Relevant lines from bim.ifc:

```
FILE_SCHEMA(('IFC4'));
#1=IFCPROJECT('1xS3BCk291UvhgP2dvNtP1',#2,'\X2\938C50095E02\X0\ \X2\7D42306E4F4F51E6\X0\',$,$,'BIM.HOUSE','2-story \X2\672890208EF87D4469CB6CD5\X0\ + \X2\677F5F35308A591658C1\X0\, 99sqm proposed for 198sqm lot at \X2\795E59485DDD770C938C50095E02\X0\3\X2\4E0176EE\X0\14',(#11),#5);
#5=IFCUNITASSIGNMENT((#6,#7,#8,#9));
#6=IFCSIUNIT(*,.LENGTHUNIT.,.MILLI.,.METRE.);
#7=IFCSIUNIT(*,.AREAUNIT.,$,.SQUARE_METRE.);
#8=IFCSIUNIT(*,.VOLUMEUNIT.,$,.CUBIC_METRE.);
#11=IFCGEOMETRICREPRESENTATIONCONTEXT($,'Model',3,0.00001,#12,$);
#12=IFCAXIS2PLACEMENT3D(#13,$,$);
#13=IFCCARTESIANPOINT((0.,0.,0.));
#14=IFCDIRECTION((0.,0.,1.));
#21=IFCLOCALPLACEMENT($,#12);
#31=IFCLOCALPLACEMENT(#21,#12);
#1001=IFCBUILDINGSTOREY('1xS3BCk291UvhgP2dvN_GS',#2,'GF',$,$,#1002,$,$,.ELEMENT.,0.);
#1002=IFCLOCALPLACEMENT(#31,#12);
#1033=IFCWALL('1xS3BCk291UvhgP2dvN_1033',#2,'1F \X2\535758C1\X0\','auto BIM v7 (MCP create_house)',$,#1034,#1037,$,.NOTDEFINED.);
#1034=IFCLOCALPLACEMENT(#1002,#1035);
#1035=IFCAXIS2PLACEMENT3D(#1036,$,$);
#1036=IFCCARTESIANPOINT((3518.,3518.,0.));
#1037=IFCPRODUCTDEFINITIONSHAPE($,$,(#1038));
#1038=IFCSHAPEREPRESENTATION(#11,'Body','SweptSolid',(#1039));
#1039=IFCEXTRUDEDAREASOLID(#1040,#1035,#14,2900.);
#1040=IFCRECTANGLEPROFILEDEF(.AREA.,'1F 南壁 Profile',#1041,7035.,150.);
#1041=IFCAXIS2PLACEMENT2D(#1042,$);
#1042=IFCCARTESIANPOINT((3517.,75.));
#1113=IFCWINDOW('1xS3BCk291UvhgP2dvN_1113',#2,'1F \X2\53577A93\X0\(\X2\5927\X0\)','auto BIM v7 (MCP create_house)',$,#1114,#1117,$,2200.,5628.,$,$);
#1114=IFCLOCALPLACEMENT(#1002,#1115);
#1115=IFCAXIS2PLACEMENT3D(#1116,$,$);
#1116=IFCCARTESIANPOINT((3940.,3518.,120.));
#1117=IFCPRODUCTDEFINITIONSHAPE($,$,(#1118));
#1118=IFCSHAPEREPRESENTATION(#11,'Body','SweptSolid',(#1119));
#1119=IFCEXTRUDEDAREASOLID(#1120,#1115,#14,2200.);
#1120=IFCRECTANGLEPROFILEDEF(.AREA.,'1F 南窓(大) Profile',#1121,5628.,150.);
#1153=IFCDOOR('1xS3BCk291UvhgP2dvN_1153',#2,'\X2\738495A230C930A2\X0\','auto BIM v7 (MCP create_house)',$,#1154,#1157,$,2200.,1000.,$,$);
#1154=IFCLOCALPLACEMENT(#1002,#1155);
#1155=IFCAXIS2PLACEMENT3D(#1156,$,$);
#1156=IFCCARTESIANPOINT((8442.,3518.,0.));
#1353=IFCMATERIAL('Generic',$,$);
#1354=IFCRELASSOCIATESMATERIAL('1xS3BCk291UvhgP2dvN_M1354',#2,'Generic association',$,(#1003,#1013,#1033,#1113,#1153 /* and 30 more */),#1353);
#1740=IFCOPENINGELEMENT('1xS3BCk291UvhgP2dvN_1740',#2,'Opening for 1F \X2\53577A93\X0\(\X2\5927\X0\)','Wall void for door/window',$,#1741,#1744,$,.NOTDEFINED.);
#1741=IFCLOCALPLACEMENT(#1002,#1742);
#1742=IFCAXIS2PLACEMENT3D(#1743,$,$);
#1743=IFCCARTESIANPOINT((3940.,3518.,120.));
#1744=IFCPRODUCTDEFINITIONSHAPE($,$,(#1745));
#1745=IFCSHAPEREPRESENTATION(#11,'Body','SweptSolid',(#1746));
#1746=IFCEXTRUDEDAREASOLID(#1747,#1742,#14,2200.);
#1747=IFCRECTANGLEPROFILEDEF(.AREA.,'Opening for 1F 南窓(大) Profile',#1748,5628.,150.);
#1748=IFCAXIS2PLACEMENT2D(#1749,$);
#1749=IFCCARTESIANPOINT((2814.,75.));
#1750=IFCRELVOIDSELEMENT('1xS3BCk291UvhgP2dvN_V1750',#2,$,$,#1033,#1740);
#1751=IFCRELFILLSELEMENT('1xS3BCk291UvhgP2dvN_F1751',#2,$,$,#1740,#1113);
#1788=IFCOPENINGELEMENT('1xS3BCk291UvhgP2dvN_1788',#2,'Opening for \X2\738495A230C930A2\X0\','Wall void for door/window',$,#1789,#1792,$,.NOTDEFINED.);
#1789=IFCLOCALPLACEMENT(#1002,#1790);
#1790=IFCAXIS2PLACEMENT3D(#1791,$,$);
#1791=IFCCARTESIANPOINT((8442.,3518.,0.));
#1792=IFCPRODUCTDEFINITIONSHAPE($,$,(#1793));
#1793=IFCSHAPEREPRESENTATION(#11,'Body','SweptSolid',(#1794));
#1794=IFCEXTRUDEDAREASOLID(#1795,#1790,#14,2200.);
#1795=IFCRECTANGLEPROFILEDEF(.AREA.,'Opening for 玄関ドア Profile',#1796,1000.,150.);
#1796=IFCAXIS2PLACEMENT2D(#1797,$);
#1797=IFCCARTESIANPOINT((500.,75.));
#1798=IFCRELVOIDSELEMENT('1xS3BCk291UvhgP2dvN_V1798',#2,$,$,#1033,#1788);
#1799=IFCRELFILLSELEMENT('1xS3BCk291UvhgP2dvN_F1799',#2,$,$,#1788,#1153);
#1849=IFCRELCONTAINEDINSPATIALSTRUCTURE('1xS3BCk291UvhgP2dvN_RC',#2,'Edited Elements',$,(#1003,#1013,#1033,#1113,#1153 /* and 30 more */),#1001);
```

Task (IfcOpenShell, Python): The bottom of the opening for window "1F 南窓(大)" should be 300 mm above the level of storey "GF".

```python
import numpy as np
import ifcopenshell
import ifcopenshell.api.geometry
import ifcopenshell.geom
import ifcopenshell.util.element
import ifcopenshell.util.placement
import ifcopenshell.util.shape
import ifcopenshell.util.unit

model = ifcopenshell.open("bim.ifc")
unit_scale = ifcopenshell.util.unit.calculate_unit_scale(model)

window = model.by_guid("1xS3BCk291UvhgP2dvN_1113")
opening = window.FillsVoids[0].RelatingOpeningElement
storey = ifcopenshell.util.element.get_container(window, ifc_class="IfcBuildingStorey")
level = ifcopenshell.util.placement.get_local_placement(storey.ObjectPlacement)[2, 3]

# The opening's origin need not be at the sill, so measure its lowest point.
shape = ifcopenshell.geom.create_shape(ifcopenshell.geom.settings(), opening)
bottom = ifcopenshell.util.shape.get_shape_bottom_elevation(shape, shape.geometry) / unit_scale
dz = level + 0.3 / unit_scale - bottom

shift = np.array([0.0, 0.0, dz])
# The window is not placed relative to its opening, so move both.
for product in (opening, window):
    matrix = ifcopenshell.util.placement.get_local_placement(product.ObjectPlacement)
    matrix[:3, 3] += shift
    ifcopenshell.api.geometry.edit_object_placement(model, product=product, matrix=matrix, is_si=False)

print(f"moved by {dz * unit_scale:+.3f} m")

model.write("bim_updated.ifc")
```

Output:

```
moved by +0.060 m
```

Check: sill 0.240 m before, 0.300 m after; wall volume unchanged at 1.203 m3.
